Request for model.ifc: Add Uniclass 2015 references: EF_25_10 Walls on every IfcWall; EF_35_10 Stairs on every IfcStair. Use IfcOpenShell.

First a look at what the model holds.

```python
import ifcopenshell

model = ifcopenshell.open("model.ifc")
print(model.schema)
print("classifications:", [c.Name for c in model.by_type("IfcClassification")])
for ifc_class in ("IfcDoor", "IfcRoof", "IfcStair", "IfcWall", "IfcWindow"):
    print(ifc_class, len(model.by_type(ifc_class)))
```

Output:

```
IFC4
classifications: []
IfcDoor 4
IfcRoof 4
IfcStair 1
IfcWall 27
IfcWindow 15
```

```python
import ifcopenshell
import ifcopenshell.api.classification

model = ifcopenshell.open("model.ifc")

system = ifcopenshell.api.classification.add_classification(model, classification="Uniclass 2015")

codes = {
    "IfcWall": ("EF_25_10", "Walls"),
    "IfcStair": ("EF_35_10", "Stairs"),
}
for ifc_class, (code, name) in codes.items():
    products = model.by_type(ifc_class)
    ifcopenshell.api.classification.add_reference(
        model, products=products, classification=system, identification=code, name=name
    )
    print(code, len(products))

model.write("model_rev.ifc")
```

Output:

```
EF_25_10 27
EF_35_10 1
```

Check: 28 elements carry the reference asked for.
